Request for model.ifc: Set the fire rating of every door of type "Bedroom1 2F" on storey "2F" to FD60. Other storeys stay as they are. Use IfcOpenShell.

First a look at what the model holds.

```python
import ifcopenshell
import ifcopenshell.util.element

model = ifcopenshell.open("model.ifc")
print(model.schema)
storey = next(s for s in model.by_type("IfcBuildingStorey") if s.Name == "2F")
doors = [e for e in ifcopenshell.util.element.get_decomposition(storey) if e.is_a("IfcDoor")]
seen = {}
for e in doors:
    element_type = ifcopenshell.util.element.get_type(e)
    key = (element_type.Name if element_type != e and element_type else None, ifcopenshell.util.element.get_pset(e, "Pset_DoorCommon", "FireRating"))
    seen[key] = seen.get(key, 0) + 1
for (name, value), count in sorted(seen.items(), key=str):
    print(count, "x", name, "|", value)
```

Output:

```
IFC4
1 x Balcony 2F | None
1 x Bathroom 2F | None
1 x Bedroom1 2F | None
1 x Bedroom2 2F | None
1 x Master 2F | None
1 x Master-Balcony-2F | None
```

```python
import ifcopenshell
import ifcopenshell.api.pset
import ifcopenshell.util.element

model = ifcopenshell.open("model.ifc")

storey = next(s for s in model.by_type("IfcBuildingStorey") if s.Name == "2F")
doors = [e for e in ifcopenshell.util.element.get_decomposition(storey) if e.is_a("IfcDoor")]

count = 0
for e in doors:
    element_type = ifcopenshell.util.element.get_type(e)
    if element_type in (None, e) or element_type.Name != "Bedroom1 2F":
        continue
    # add_pset returns the element's existing set when there is one.
    pset = ifcopenshell.api.pset.add_pset(model, product=e, name="Pset_DoorCommon")
    ifcopenshell.api.pset.edit_pset(model, pset=pset, properties={"FireRating": "FD60"})
    count += 1

print(count, "doors updated")

model.write("model_edited.ifc")
```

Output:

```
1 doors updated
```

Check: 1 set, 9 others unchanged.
